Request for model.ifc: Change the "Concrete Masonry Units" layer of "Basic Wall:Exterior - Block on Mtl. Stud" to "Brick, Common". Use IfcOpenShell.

First a look at what the model holds.

```python
import ifcopenshell
import ifcopenshell.util.element

model = ifcopenshell.open("model.ifc")
print(model.schema)
for layer_set in model.by_type("IfcMaterialLayerSet"):
    if layer_set.LayerSetName == "Basic Wall:Exterior - Block on Mtl. Stud":
        for layer in layer_set.MaterialLayers:
            print(layer.id(), layer.Material and layer.Material.Name, layer.LayerThickness, sep=" | ")
        print(len(ifcopenshell.util.element.get_elements_by_material(model, layer_set)), "elements and types use it")
print(sorted(m.Name for m in model.by_type("IfcMaterial") if m.Name)[:60])
```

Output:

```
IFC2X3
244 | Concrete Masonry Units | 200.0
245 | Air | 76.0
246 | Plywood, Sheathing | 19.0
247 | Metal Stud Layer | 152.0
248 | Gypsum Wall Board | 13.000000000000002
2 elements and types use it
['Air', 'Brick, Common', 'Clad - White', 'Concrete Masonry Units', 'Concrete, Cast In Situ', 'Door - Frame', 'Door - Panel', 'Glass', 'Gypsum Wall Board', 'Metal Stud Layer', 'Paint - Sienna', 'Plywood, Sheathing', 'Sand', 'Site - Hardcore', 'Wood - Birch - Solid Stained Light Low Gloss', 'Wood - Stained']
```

```python
import ifcopenshell
import ifcopenshell.api.material

model = ifcopenshell.open("model.ifc")

layer_set = next(s for s in model.by_type("IfcMaterialLayerSet") if s.LayerSetName == "Basic Wall:Exterior - Block on Mtl. Stud")
layer = next(l for l in layer_set.MaterialLayers if l.Material and l.Material.Name == "Concrete Masonry Units")
material = next(m for m in model.by_type("IfcMaterial") if m.Name == "Brick, Common")

# Point this one layer at the other material; renaming the old one would change it everywhere.
ifcopenshell.api.material.edit_layer(model, layer=layer, attributes={}, material=material)

print([l.Material.Name if l.Material else None for l in layer_set.MaterialLayers])

model.write("model_updated.ifc")
```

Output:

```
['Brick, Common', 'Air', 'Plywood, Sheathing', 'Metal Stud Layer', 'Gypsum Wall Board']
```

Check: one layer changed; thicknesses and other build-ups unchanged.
